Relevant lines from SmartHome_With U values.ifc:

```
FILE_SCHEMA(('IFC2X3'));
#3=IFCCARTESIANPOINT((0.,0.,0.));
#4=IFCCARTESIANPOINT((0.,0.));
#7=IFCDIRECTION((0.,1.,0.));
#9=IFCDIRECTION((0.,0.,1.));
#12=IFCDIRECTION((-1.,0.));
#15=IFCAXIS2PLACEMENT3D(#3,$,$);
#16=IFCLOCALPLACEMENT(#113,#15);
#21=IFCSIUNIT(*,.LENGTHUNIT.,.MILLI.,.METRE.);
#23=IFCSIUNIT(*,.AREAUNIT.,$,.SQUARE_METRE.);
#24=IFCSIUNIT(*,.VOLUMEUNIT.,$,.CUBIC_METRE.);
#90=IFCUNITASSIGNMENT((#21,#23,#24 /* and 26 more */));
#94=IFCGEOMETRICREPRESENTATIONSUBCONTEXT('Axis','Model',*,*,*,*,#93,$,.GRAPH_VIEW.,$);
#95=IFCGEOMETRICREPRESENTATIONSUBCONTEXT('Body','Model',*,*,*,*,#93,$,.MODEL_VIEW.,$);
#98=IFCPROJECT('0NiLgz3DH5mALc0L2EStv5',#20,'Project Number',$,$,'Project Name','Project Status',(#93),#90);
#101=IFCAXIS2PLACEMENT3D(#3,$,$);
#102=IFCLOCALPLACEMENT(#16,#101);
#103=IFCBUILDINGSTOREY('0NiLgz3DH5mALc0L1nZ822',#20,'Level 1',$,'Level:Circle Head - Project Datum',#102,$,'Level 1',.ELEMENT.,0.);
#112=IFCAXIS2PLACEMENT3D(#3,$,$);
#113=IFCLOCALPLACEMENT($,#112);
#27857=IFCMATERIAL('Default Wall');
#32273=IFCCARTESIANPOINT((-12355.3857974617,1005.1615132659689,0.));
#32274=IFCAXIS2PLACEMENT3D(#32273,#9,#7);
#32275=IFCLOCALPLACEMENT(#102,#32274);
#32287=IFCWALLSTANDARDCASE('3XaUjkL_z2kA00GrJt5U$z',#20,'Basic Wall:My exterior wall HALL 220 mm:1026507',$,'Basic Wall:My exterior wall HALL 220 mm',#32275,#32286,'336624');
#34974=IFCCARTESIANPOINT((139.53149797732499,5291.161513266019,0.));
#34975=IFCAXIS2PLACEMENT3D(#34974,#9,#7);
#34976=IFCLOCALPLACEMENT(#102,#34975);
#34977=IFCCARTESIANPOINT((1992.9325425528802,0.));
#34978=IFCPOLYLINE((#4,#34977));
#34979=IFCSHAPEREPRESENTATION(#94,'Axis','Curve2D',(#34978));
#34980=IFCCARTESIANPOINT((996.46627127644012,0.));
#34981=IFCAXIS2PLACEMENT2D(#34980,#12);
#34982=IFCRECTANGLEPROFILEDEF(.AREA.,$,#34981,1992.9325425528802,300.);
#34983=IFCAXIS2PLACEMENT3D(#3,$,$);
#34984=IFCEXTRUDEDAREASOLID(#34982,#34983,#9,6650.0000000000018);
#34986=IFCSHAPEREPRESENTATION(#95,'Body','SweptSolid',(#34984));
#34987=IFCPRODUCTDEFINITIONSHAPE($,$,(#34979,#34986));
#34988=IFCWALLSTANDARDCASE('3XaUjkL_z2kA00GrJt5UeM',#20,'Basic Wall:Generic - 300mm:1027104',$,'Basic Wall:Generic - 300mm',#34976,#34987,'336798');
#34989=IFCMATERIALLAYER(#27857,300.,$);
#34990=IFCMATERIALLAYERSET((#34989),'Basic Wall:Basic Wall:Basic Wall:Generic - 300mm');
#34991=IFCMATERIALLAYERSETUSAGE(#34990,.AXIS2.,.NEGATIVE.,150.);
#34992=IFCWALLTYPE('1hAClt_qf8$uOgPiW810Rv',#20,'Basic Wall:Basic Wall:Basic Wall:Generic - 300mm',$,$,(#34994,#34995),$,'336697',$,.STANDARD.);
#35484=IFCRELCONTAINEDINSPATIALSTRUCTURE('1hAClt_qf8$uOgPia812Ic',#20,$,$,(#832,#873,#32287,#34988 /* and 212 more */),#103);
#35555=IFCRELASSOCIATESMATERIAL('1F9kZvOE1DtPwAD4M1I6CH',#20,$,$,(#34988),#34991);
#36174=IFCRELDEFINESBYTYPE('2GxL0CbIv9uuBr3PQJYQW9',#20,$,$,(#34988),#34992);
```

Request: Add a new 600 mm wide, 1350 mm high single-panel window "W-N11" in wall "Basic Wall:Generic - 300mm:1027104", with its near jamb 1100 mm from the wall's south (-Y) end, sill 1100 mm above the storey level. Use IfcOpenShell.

```python
import numpy as np
import ifcopenshell
import ifcopenshell.api.feature
import ifcopenshell.api.geometry
import ifcopenshell.api.root
import ifcopenshell.api.spatial
import ifcopenshell.api.type
import ifcopenshell.geom
import ifcopenshell.util.element
import ifcopenshell.util.placement
import ifcopenshell.util.representation
import ifcopenshell.util.shape
import ifcopenshell.util.unit

model = ifcopenshell.open("SmartHome_With U values.ifc")
unit_scale = ifcopenshell.util.unit.calculate_unit_scale(model)
settings = ifcopenshell.geom.settings()


def volume(element):
    """Net volume in cubic metres, openings subtracted."""
    shape = ifcopenshell.geom.create_shape(settings, element)
    return ifcopenshell.util.shape.get_volume(shape.geometry)


wall = model.by_guid("3XaUjkL_z2kA00GrJt5UeM")
storey = ifcopenshell.util.element.get_container(wall, ifc_class="IfcBuildingStorey")
context = ifcopenshell.util.representation.get_context(model, "Model", "Body", "MODEL_VIEW")
before = volume(wall)

width, height, from_end, sill = 0.6, 1.35, 1.1, 1.1  # metres

# The wall runs along its own X axis, and the end named is its -X end.
wall_shape = ifcopenshell.geom.create_shape(settings, wall)
x, y, z = ifcopenshell.util.shape.get_vertices(wall_shape.geometry).T
start = x.min() + from_end
face, thickness = float(y.min()), float(y.max() - y.min())
wall_matrix = ifcopenshell.util.placement.get_local_placement(wall.ObjectPlacement)
level = ifcopenshell.util.placement.get_local_placement(storey.ObjectPlacement)[2, 3]


def in_wall(x, y):
    """Placement at x, y metres in the wall's axes, at sill height."""
    matrix = wall_matrix.copy()
    matrix[:, 3] = wall_matrix @ np.array([x / unit_scale, y / unit_scale, 0.0, 1.0])
    matrix[2, 3] = level + sill / unit_scale
    return matrix


# Opening: a box that overshoots both wall faces by 50 mm.
opening = ifcopenshell.api.root.create_entity(model, ifc_class="IfcOpeningElement")
box = ifcopenshell.api.geometry.add_wall_representation(
    model, context=context, length=width, height=height, thickness=thickness + 0.1
)
ifcopenshell.api.geometry.assign_representation(model, product=opening, representation=box)
ifcopenshell.api.geometry.edit_object_placement(model, product=opening, matrix=in_wall(start, face - 0.05), is_si=False)
ifcopenshell.api.feature.add_feature(model, feature=opening, element=wall)

window = ifcopenshell.api.root.create_entity(model, ifc_class="IfcWindow", name="W-N11")
window.OverallWidth, window.OverallHeight = width / unit_scale, height / unit_scale
body = ifcopenshell.api.geometry.add_window_representation(
    model,
    context=context,
    overall_width=window.OverallWidth,
    overall_height=window.OverallHeight,
    partition_type="SINGLE_PANEL",
)
ifcopenshell.api.geometry.assign_representation(model, product=window, representation=body)
ifcopenshell.api.spatial.assign_container(model, products=[window], relating_structure=storey)
fills = ifcopenshell.api.feature.add_filling(model, opening=opening, element=window)
fills.OwnerHistory = window.OwnerHistory  # required in IFC2X3

# IFC2X3 keeps the operation on the window style.
style = ifcopenshell.api.root.create_entity(model, ifc_class="IfcWindowStyle", name="W-N11")
style.OperationType, style.ConstructionType = "SINGLE_PANEL", "NOTDEFINED"
style.ParameterTakesPrecedence = style.Sizeable = False
ifcopenshell.api.type.assign_type(model, related_objects=[window], relating_type=style)

# Centre the window in the wall's thickness.
ifcopenshell.api.geometry.edit_object_placement(model, product=window, matrix=in_wall(start, face), is_si=False)
window_shape = ifcopenshell.geom.create_shape(settings, window)
depth = ifcopenshell.util.shape.get_vertices(window_shape.geometry)[:, 1]
offset = face + thickness / 2 - (depth.min() + depth.max()) / 2
ifcopenshell.api.geometry.edit_object_placement(model, product=window, matrix=in_wall(start, offset), is_si=False)

after = volume(wall)

print(f"wall volume {before:.3f} -> {after:.3f} m3")

model.write("SmartHome_With U values-out.ifc")
```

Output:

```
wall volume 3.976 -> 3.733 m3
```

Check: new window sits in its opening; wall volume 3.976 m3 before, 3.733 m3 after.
